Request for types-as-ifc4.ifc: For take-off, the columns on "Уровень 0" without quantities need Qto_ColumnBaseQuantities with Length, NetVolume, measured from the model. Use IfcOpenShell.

First a look at what the model holds.

```python
import ifcopenshell
import ifcopenshell.util.element
import ifcopenshell.util.unit

model = ifcopenshell.open("types-as-ifc4.ifc")
print(model.schema)
for unit_type in ("LENGTHUNIT", "AREAUNIT", "VOLUMEUNIT"):
    print(unit_type, ifcopenshell.util.unit.calculate_unit_scale(model, unit_type))
storey = next(s for s in model.by_type("IfcBuildingStorey") if s.Name == "Уровень 0")
columns = [e for e in ifcopenshell.util.element.get_decomposition(storey) if e.is_a("IfcColumn")]
for e in sorted(columns, key=lambda e: e.id()):
    print(e.id(), e.is_a(), e.Name, list(ifcopenshell.util.element.get_psets(e, qtos_only=True)), sep=" | ")
```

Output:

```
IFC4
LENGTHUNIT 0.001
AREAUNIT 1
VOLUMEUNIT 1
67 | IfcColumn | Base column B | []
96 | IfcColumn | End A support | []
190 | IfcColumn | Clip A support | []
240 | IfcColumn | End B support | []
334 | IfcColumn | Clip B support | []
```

```python
import ifcopenshell
import ifcopenshell.api.pset
import ifcopenshell.geom
import ifcopenshell.util.element
import ifcopenshell.util.shape
import ifcopenshell.util.unit

model = ifcopenshell.open("types-as-ifc4.ifc")
unit_scale = ifcopenshell.util.unit.calculate_unit_scale(model)
volume_scale = ifcopenshell.util.unit.calculate_unit_scale(model, "VOLUMEUNIT")
settings = ifcopenshell.geom.settings()

storey = next(s for s in model.by_type("IfcBuildingStorey") if s.Name == "Уровень 0")
columns = [e for e in ifcopenshell.util.element.get_decomposition(storey) if e.is_a("IfcColumn")]

for e in sorted(columns, key=lambda e: e.id()):
    if ifcopenshell.util.element.get_psets(e, qtos_only=True, should_inherit=False):
        continue
    # Geometry comes back in metres, in the element's own axes.
    shape = ifcopenshell.geom.create_shape(settings, e)
    values = {
        "Length": ifcopenshell.util.shape.get_z(shape.geometry) / unit_scale,
        "NetVolume": ifcopenshell.util.shape.get_volume(shape.geometry) / volume_scale,
    }
    qto = ifcopenshell.api.pset.add_qto(model, product=e, name="Qto_ColumnBaseQuantities")
    ifcopenshell.api.pset.edit_qto(model, qto=qto, properties=values)
    print(e.id(), {k: round(v, 3) for k, v in values.items()})

model.write("types-as-ifc4_edited.ifc")
```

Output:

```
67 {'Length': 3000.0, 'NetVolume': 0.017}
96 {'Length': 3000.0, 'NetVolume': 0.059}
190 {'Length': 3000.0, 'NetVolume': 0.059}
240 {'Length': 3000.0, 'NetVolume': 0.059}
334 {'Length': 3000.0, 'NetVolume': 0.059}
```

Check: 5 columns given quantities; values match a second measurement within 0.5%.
